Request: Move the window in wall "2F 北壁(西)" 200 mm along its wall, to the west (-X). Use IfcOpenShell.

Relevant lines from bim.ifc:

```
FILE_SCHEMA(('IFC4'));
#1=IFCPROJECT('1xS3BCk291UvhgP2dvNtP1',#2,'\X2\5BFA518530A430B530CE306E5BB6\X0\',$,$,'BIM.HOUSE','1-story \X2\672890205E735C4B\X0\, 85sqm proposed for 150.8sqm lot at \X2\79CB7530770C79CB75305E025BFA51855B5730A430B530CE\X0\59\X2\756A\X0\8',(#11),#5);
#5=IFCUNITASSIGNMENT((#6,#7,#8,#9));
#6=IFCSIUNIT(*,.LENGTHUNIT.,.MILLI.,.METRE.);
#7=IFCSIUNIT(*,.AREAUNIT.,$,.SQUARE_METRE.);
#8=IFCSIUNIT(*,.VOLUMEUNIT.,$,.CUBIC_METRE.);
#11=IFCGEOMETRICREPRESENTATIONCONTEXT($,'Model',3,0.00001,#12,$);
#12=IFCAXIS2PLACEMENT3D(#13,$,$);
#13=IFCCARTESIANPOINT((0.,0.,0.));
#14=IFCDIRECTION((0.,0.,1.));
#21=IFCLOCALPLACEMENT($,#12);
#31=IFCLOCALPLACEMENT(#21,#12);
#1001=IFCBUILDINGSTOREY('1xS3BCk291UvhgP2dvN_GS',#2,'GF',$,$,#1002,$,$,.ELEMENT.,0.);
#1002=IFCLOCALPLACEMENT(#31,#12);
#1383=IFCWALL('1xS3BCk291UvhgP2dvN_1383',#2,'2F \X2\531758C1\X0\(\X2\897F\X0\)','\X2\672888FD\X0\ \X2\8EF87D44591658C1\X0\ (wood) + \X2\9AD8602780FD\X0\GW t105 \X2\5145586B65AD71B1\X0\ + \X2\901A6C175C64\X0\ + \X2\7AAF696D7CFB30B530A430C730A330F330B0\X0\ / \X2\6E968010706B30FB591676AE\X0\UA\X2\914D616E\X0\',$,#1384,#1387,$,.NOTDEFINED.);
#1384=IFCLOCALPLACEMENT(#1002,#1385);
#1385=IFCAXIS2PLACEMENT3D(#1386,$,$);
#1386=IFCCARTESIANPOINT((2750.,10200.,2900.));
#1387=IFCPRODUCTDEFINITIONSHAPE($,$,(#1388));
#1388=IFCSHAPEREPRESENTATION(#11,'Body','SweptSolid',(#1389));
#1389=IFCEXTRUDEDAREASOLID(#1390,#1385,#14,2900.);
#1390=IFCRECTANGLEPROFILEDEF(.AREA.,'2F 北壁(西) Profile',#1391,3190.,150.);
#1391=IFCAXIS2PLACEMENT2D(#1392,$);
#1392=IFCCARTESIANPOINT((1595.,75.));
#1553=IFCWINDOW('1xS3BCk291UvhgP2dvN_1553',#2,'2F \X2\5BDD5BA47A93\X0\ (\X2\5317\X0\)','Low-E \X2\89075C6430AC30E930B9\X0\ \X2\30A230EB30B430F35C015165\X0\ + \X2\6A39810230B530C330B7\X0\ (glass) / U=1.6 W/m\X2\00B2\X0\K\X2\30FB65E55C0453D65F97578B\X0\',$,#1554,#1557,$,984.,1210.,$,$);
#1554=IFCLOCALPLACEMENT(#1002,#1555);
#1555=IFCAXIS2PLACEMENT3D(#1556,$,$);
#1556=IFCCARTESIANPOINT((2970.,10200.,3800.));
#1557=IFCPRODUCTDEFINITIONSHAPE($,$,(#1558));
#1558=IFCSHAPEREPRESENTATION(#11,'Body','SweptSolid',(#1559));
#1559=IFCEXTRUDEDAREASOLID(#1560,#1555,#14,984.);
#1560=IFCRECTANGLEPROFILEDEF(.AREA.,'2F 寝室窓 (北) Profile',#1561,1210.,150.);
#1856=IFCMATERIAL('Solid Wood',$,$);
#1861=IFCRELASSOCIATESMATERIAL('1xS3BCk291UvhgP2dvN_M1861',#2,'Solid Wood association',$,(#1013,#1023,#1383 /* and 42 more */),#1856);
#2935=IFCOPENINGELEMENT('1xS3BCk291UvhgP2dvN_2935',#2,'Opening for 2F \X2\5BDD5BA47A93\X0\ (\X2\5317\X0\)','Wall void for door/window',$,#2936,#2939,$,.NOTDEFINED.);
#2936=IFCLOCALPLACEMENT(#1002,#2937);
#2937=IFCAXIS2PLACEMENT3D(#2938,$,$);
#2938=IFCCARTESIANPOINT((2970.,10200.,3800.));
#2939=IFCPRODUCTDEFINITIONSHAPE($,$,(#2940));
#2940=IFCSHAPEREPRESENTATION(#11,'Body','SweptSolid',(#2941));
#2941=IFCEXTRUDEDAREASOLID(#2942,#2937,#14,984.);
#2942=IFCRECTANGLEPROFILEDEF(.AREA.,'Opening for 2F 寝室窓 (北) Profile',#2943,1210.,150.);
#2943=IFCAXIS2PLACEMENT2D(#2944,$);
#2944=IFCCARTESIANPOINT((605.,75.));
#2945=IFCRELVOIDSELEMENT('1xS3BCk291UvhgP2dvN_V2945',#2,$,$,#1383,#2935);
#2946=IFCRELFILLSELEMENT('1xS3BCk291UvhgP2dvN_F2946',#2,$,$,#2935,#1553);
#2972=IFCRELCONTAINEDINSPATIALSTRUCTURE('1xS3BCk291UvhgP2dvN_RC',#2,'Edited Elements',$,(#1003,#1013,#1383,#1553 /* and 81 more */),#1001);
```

```python
import ifcopenshell
import ifcopenshell.api.geometry
import ifcopenshell.util.placement
import ifcopenshell.util.unit

model = ifcopenshell.open("bim.ifc")
unit_scale = ifcopenshell.util.unit.calculate_unit_scale(model)

window = model.by_guid("1xS3BCk291UvhgP2dvN_1553")
opening = window.FillsVoids[0].RelatingOpeningElement
wall = opening.VoidsElements[0].RelatingBuildingElement

wall_matrix = ifcopenshell.util.placement.get_local_placement(wall.ObjectPlacement)
shift = wall_matrix[:3, 0] * -0.2 / unit_scale
before = ifcopenshell.util.placement.get_local_placement(window.ObjectPlacement)[:3, 3].copy()

# The window is not placed relative to its opening, so move both.
for product in (opening, window):
    matrix = ifcopenshell.util.placement.get_local_placement(product.ObjectPlacement)
    matrix[:3, 3] += shift
    ifcopenshell.api.geometry.edit_object_placement(model, product=product, matrix=matrix, is_si=False)

after = ifcopenshell.util.placement.get_local_placement(window.ObjectPlacement)[:3, 3]
print("window moved by", (after - before).round(3) + 0.0)

model.write("bim_edited.ifc")
```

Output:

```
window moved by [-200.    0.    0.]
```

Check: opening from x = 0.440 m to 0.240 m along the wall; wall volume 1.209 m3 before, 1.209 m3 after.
